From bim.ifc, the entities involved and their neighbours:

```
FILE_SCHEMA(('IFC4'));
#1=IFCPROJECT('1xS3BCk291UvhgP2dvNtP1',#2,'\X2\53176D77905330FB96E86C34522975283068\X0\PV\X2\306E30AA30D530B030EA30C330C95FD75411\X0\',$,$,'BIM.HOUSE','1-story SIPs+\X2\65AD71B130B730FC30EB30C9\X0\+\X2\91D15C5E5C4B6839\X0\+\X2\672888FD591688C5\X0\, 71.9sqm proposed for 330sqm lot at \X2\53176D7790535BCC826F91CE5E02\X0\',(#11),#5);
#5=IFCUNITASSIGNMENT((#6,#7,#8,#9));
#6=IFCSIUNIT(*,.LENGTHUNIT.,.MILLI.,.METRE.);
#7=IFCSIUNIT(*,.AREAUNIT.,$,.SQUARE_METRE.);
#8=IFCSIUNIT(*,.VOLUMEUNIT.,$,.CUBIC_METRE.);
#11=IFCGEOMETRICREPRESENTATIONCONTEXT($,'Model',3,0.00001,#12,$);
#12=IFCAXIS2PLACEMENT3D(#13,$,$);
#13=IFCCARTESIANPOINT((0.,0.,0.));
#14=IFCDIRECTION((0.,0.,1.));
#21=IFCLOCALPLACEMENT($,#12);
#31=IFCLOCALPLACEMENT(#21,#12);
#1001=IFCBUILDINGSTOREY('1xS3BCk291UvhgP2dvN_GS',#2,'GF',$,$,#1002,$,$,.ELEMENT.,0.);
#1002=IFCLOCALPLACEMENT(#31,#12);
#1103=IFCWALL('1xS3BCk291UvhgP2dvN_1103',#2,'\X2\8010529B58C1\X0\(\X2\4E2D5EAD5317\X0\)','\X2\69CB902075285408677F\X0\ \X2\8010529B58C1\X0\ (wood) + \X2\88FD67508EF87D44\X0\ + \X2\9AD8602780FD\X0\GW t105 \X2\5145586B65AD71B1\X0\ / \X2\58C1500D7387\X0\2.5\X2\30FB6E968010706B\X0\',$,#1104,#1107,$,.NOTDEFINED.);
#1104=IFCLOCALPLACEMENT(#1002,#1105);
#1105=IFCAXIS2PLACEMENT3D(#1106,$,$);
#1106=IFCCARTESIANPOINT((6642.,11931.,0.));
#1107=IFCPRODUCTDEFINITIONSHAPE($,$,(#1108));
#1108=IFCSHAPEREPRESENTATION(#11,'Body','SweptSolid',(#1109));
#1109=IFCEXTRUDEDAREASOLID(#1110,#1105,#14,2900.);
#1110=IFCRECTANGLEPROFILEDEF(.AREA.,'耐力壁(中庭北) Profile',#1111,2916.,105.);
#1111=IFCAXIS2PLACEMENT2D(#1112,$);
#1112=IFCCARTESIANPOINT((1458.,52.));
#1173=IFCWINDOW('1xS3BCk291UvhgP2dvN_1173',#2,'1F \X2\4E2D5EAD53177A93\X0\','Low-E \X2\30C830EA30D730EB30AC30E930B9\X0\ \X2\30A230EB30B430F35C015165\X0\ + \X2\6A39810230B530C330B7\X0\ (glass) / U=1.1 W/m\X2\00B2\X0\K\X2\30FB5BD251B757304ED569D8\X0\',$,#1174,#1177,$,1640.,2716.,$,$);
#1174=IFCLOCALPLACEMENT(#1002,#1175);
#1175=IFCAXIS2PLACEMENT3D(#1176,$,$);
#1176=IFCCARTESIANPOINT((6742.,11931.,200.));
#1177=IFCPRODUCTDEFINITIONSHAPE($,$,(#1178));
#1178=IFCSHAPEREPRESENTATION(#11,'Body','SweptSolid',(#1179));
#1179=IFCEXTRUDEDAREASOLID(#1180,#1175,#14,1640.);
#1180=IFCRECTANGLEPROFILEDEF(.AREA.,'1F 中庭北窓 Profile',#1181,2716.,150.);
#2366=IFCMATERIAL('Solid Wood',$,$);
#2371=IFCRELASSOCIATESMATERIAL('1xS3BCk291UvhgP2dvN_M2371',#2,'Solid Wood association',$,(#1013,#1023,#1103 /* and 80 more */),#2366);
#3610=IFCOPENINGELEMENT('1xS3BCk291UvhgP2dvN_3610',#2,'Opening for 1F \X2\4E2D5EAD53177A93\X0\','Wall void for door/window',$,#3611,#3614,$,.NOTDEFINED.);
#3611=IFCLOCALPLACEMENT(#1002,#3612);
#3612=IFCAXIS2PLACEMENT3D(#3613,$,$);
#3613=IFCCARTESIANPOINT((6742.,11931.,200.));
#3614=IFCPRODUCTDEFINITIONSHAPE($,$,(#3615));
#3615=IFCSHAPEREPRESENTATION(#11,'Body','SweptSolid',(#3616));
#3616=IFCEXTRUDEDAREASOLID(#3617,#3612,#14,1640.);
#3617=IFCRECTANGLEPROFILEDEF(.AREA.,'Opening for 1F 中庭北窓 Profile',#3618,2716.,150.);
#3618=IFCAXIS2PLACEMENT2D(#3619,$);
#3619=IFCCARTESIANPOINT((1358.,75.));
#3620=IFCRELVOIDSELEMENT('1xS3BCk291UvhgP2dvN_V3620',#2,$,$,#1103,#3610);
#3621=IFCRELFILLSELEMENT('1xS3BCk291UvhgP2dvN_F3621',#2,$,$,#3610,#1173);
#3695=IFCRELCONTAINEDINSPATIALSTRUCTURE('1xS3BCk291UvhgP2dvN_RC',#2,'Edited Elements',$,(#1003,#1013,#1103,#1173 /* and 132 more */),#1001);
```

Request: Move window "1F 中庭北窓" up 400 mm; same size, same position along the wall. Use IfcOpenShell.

```python
import numpy as np
import ifcopenshell
import ifcopenshell.api.geometry
import ifcopenshell.util.placement
import ifcopenshell.util.unit

model = ifcopenshell.open("bim.ifc")
unit_scale = ifcopenshell.util.unit.calculate_unit_scale(model)

window = model.by_id(1173)
opening = window.FillsVoids[0].RelatingOpeningElement
dz = 400.0

shift = np.array([0.0, 0.0, dz])
# The window is not placed relative to its opening, so move both.
for product in (opening, window):
    matrix = ifcopenshell.util.placement.get_local_placement(product.ObjectPlacement)
    matrix[:3, 3] += shift
    ifcopenshell.api.geometry.edit_object_placement(model, product=product, matrix=matrix, is_si=False)

print(f"moved by {dz * unit_scale:+.3f} m")

model.write("bim_rev.ifc")
```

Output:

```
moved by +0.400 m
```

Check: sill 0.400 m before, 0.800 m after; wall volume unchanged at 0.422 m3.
